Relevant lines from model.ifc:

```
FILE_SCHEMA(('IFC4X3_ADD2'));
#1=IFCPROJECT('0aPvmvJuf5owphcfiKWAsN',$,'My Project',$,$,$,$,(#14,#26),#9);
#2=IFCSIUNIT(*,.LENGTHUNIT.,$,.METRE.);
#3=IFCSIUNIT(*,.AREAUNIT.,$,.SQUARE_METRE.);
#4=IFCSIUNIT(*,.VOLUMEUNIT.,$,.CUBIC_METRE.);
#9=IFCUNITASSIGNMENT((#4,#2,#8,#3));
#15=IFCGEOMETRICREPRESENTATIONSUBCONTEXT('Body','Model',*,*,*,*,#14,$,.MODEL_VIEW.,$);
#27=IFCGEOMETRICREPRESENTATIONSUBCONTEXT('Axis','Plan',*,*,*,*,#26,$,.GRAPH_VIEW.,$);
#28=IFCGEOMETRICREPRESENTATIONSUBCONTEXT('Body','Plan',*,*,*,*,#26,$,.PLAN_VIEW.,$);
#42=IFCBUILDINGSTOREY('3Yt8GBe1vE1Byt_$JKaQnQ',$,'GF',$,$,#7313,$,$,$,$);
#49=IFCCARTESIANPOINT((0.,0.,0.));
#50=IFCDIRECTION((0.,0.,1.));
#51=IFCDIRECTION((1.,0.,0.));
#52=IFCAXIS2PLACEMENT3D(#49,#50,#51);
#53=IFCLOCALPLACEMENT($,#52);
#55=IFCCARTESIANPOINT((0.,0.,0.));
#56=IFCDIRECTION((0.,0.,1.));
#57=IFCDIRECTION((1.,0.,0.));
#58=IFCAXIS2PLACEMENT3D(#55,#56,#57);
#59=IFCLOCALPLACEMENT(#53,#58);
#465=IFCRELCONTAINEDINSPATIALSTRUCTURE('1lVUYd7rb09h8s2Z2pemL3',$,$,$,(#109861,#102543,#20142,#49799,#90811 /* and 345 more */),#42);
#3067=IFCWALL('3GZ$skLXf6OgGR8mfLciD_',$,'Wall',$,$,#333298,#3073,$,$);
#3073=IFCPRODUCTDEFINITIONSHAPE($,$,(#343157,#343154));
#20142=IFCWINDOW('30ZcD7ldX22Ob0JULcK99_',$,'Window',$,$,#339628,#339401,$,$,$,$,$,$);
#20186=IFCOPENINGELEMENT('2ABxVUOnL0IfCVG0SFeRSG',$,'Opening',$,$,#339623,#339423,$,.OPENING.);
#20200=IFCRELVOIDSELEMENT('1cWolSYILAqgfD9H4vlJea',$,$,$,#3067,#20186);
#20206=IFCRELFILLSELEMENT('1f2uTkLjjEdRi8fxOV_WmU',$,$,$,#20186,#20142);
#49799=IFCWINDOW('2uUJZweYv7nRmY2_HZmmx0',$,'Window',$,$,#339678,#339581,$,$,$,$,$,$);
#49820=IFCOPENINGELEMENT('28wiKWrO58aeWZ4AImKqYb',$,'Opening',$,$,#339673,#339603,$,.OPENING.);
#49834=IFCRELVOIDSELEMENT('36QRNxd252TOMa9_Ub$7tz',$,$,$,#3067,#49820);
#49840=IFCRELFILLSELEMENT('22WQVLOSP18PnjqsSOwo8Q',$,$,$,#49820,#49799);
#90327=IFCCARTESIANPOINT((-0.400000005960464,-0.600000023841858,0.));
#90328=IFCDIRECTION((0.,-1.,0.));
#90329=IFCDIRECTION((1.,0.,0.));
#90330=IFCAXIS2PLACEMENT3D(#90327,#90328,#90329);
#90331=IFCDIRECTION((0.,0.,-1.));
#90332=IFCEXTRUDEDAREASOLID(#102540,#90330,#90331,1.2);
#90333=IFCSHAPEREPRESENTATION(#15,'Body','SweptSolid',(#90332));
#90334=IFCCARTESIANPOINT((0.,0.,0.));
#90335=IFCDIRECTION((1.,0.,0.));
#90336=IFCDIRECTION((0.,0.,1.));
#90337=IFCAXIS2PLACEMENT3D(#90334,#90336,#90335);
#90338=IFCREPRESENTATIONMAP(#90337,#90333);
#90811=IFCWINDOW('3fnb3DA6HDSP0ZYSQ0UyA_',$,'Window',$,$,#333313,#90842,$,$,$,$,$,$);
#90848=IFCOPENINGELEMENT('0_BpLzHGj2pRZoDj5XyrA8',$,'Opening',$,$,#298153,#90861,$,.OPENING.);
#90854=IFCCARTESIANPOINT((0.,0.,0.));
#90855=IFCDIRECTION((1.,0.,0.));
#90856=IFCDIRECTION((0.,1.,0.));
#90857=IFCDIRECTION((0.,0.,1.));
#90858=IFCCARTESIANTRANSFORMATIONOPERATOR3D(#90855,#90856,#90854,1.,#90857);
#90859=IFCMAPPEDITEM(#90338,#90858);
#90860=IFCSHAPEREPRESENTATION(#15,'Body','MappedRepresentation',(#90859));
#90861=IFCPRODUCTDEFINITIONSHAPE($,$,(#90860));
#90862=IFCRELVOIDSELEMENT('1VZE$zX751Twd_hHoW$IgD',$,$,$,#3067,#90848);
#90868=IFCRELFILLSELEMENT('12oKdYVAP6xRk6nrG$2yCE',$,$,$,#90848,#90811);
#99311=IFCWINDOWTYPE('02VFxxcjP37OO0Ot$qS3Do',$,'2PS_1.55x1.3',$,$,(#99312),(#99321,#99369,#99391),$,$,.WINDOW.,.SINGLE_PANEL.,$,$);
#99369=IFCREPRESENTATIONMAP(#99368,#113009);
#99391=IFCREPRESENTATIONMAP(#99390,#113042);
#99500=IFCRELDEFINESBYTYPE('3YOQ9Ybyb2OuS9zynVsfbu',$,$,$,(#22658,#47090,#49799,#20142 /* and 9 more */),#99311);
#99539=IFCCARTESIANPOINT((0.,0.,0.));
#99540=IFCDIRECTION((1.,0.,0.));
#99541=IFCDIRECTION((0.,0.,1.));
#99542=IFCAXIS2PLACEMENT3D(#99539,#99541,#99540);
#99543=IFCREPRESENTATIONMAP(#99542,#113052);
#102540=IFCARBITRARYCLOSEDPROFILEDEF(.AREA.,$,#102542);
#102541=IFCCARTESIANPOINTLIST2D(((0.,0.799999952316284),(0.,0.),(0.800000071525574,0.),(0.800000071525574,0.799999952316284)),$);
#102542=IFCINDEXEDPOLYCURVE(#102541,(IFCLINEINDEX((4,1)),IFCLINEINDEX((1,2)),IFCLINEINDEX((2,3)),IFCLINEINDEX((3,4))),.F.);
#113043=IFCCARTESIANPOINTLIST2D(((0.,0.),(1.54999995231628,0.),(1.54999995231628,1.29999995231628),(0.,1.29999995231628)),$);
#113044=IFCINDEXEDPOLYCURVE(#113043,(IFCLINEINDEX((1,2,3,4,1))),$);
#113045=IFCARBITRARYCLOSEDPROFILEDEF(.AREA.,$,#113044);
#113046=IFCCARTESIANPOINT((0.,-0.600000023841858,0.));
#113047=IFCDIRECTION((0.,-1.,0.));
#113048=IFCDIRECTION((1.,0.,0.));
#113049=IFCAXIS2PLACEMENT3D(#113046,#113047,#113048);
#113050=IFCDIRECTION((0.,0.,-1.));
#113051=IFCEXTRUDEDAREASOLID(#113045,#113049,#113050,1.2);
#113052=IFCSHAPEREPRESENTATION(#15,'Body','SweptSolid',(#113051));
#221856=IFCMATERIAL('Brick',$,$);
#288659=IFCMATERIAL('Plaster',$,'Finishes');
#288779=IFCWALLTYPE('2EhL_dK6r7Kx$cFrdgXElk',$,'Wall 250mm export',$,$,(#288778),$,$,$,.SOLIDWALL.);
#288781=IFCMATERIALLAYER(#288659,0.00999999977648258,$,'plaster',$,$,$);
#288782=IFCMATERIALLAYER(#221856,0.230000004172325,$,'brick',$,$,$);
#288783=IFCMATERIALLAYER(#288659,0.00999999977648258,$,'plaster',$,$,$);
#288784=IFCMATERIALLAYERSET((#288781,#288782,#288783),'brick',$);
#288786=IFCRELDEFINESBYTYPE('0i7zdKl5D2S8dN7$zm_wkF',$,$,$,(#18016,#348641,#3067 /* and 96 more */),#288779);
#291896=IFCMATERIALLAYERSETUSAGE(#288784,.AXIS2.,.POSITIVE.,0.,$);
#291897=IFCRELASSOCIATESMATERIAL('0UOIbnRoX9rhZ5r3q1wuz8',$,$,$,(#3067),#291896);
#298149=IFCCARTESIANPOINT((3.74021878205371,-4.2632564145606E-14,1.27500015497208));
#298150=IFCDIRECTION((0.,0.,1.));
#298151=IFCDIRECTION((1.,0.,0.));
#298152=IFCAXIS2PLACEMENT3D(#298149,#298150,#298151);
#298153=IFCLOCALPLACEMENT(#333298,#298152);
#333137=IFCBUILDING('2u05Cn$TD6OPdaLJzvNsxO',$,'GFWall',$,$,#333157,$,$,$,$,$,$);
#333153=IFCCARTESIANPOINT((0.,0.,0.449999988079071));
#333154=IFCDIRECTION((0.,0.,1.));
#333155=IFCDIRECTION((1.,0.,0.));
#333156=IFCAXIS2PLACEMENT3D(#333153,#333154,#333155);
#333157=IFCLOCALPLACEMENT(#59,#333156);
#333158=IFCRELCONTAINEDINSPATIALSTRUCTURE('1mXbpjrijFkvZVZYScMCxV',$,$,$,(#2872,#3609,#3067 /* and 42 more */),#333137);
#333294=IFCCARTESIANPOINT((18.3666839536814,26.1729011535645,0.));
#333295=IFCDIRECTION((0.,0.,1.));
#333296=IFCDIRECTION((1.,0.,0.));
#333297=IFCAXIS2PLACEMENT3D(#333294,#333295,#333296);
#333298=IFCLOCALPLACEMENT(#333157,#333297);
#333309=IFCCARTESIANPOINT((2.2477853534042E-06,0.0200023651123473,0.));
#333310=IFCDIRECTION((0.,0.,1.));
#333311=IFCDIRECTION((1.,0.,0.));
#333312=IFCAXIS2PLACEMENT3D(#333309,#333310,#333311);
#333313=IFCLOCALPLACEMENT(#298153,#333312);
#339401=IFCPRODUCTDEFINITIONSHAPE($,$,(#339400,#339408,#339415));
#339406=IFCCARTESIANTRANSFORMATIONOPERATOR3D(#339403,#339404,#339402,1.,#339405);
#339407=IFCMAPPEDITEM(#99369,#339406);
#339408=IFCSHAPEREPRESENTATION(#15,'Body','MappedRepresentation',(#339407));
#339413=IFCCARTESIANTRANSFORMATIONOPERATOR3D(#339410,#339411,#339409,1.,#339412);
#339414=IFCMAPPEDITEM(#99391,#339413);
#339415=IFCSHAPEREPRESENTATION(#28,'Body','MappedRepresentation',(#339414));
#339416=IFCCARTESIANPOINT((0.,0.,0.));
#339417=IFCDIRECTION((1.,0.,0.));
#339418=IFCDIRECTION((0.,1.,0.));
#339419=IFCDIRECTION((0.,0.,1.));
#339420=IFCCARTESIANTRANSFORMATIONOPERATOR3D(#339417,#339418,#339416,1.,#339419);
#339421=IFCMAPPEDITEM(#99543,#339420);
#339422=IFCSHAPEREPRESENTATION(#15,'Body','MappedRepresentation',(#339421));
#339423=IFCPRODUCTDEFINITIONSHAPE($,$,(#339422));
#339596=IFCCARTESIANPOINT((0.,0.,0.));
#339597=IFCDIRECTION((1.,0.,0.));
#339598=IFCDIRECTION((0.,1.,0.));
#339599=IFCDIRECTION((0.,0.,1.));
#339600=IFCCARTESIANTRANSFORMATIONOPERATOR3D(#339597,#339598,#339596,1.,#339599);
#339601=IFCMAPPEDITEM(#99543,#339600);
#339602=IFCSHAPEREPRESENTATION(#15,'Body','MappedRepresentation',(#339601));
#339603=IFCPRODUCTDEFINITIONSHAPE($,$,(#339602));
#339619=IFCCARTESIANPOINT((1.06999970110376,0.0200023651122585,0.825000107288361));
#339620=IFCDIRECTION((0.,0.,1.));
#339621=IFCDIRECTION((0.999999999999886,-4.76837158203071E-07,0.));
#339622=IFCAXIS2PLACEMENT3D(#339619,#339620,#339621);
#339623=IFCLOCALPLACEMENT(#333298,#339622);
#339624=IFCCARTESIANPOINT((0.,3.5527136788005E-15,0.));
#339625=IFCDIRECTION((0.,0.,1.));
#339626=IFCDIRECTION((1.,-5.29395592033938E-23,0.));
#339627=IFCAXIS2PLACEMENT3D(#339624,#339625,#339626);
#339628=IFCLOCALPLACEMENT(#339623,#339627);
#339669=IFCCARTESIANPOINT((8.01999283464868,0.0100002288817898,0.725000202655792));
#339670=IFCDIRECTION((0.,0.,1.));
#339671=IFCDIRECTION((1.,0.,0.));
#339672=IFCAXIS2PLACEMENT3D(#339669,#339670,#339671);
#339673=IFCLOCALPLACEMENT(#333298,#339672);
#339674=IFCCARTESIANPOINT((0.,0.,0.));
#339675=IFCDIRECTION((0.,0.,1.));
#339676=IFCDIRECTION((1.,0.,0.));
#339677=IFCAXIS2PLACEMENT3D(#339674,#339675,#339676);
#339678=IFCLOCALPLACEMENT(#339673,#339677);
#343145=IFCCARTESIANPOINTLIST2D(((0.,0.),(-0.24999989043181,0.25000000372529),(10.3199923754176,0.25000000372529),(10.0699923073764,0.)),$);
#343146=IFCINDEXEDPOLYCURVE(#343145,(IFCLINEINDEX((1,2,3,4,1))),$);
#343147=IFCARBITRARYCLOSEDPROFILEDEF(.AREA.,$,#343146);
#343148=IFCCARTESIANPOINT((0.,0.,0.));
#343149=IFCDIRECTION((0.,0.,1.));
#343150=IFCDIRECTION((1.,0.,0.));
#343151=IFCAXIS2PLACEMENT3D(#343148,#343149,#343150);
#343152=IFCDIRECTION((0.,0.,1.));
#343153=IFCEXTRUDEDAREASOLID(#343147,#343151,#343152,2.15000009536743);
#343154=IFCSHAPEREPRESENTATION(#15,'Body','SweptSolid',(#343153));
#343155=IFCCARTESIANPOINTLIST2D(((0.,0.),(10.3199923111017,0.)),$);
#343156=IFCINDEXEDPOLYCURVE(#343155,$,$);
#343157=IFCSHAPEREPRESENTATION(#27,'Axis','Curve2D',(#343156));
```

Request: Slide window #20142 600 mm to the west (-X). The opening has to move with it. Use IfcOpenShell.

```python
import ifcopenshell
import ifcopenshell.api.geometry
import ifcopenshell.util.placement
import ifcopenshell.util.unit

model = ifcopenshell.open("model.ifc")
unit_scale = ifcopenshell.util.unit.calculate_unit_scale(model)

window = model.by_guid("30ZcD7ldX22Ob0JULcK99_")
opening = window.FillsVoids[0].RelatingOpeningElement
wall = opening.VoidsElements[0].RelatingBuildingElement

wall_matrix = ifcopenshell.util.placement.get_local_placement(wall.ObjectPlacement)
shift = wall_matrix[:3, 0] * -0.6 / unit_scale
before = ifcopenshell.util.placement.get_local_placement(window.ObjectPlacement)[:3, 3].copy()

# The window is placed relative to its opening, so it follows when the opening moves.
matrix = ifcopenshell.util.placement.get_local_placement(opening.ObjectPlacement)
matrix[:3, 3] += shift
ifcopenshell.api.geometry.edit_object_placement(
    model, product=opening, matrix=matrix, is_si=False, should_transform_children=True
)

after = ifcopenshell.util.placement.get_local_placement(window.ObjectPlacement)[:3, 3]
print("window moved by", (after - before).round(3) + 0.0)

model.write("model_updated.ifc")
```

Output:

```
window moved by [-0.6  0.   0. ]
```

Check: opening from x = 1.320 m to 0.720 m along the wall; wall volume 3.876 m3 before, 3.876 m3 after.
